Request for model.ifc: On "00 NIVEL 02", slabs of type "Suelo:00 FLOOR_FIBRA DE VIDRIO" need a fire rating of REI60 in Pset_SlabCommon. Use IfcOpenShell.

First a look at what the model holds.

```python
import ifcopenshell
import ifcopenshell.util.element

model = ifcopenshell.open("model.ifc")
print(model.schema)
storey = next(s for s in model.by_type("IfcBuildingStorey") if s.Name == "00 NIVEL 02")
slabs = [e for e in ifcopenshell.util.element.get_decomposition(storey) if e.is_a("IfcSlab")]
seen = {}
for e in slabs:
    element_type = ifcopenshell.util.element.get_type(e)
    key = (element_type.Name if element_type != e and element_type else None, ifcopenshell.util.element.get_pset(e, "Pset_SlabCommon", "FireRating"))
    seen[key] = seen.get(key, 0) + 1
for (name, value), count in sorted(seen.items(), key=str):
    print(count, "x", name, "|", value)
```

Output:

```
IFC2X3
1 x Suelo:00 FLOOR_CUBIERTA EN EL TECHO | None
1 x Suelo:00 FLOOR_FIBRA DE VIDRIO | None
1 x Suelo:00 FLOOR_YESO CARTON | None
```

```python
import ifcopenshell
import ifcopenshell.api.pset
import ifcopenshell.util.element

model = ifcopenshell.open("model.ifc")

storey = next(s for s in model.by_type("IfcBuildingStorey") if s.Name == "00 NIVEL 02")
slabs = [e for e in ifcopenshell.util.element.get_decomposition(storey) if e.is_a("IfcSlab")]

count = 0
for e in slabs:
    element_type = ifcopenshell.util.element.get_type(e)
    if element_type in (None, e) or element_type.Name != "Suelo:00 FLOOR_FIBRA DE VIDRIO":
        continue
    # add_pset returns the element's existing set when there is one.
    pset = ifcopenshell.api.pset.add_pset(model, product=e, name="Pset_SlabCommon")
    ifcopenshell.api.pset.edit_pset(model, pset=pset, properties={"FireRating": "REI60"})
    count += 1

print(count, "slabs updated")

model.write("model_updated.ifc")
```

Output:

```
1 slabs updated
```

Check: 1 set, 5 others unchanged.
